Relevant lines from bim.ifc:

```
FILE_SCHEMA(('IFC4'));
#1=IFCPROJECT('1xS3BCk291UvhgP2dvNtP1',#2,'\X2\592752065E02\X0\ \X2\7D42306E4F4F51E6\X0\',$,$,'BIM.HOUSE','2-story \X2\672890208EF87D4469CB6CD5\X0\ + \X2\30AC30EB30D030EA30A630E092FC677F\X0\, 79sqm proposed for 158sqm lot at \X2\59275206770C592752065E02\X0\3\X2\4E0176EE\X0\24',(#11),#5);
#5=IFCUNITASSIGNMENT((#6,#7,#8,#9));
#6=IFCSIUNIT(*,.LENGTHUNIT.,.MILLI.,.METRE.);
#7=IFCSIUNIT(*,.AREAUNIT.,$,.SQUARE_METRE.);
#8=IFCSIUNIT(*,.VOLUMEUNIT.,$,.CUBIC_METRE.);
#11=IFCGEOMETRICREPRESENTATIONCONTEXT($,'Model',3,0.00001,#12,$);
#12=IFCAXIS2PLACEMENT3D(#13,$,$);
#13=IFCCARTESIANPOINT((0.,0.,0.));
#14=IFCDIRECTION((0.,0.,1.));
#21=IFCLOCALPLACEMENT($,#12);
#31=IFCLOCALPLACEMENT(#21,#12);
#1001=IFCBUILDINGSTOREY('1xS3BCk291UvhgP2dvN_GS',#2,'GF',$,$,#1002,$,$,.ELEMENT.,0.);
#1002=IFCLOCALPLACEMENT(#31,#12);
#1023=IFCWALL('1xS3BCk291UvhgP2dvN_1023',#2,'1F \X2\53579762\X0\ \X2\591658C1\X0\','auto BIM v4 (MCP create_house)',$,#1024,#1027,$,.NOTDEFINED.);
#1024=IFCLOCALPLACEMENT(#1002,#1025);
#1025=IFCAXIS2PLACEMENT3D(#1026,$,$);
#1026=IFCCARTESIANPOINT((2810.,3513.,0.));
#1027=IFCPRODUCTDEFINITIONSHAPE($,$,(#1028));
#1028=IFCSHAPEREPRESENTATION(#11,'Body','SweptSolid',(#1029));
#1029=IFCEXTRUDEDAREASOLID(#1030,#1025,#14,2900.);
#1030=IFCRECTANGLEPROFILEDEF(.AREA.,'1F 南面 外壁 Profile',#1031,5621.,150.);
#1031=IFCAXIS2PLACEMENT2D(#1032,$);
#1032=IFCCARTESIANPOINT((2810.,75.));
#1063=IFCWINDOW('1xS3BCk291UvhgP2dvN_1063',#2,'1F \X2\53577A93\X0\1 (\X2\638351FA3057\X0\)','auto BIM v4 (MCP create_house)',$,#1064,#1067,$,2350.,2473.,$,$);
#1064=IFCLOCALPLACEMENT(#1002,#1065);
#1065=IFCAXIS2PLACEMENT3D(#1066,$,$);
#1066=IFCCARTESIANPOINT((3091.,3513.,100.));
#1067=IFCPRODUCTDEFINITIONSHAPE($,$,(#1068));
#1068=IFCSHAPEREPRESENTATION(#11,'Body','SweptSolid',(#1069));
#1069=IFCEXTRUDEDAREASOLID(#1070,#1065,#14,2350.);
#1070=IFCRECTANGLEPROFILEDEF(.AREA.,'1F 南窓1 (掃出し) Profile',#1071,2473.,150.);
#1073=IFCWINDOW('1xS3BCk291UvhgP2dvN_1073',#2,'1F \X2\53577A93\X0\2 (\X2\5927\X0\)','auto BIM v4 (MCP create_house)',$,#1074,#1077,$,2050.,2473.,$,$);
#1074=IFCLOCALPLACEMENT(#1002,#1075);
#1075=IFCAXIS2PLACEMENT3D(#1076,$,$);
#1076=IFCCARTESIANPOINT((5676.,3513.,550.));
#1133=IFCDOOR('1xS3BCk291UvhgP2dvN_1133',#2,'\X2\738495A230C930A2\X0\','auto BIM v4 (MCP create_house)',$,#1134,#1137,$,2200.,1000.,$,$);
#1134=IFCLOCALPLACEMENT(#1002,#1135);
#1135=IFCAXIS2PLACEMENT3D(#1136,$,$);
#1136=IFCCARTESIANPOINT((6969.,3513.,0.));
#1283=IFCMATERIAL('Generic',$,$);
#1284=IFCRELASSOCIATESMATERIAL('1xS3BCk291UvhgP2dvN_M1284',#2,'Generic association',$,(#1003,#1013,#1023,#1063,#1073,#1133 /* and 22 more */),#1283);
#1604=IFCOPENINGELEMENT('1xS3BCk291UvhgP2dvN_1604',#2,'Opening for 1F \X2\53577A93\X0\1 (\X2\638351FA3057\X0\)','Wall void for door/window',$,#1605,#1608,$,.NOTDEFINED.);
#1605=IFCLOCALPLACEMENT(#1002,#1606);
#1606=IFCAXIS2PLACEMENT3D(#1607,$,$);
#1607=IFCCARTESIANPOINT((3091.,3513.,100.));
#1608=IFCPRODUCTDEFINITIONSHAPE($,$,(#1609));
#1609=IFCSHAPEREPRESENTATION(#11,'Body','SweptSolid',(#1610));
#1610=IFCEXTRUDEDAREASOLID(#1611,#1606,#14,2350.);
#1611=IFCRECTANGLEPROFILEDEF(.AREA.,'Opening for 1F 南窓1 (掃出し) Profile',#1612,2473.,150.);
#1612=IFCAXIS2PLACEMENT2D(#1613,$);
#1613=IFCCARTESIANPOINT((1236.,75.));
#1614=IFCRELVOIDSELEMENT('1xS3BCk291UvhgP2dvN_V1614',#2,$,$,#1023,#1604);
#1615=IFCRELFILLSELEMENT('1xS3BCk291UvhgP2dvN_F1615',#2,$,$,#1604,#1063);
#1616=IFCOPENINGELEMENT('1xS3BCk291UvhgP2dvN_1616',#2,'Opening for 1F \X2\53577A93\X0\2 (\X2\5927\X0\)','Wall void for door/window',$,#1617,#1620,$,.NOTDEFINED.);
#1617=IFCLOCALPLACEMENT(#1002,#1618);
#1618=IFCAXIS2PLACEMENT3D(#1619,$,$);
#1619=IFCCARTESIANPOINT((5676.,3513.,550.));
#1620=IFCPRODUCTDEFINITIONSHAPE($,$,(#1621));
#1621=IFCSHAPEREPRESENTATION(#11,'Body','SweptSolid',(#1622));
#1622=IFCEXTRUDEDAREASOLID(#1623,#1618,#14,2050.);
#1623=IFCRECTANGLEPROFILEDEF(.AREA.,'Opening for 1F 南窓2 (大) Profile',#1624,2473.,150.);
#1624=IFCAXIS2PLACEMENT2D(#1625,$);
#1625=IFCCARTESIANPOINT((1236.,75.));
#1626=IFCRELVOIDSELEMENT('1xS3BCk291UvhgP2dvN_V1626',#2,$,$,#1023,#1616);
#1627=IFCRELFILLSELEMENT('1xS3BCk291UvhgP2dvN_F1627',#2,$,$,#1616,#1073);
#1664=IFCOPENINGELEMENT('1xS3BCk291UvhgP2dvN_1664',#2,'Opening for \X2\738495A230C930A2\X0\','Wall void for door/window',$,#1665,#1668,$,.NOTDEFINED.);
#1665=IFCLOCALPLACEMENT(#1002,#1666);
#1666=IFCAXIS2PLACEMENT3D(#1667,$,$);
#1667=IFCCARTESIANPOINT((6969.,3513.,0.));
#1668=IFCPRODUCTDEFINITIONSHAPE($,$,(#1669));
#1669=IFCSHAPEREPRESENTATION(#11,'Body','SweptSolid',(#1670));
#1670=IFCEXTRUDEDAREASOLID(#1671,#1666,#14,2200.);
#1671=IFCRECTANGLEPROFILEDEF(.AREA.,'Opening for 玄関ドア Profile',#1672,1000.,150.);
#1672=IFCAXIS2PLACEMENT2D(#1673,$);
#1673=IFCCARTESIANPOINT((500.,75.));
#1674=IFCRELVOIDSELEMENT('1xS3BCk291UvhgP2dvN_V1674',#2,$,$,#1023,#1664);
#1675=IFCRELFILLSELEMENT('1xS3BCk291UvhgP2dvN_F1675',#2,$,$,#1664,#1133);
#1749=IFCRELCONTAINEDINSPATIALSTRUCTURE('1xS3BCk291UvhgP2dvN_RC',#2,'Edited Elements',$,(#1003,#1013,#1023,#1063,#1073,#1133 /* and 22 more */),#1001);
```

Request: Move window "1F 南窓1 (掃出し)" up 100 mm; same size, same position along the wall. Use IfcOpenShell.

```python
import numpy as np
import ifcopenshell
import ifcopenshell.api.geometry
import ifcopenshell.util.placement
import ifcopenshell.util.unit

model = ifcopenshell.open("bim.ifc")
unit_scale = ifcopenshell.util.unit.calculate_unit_scale(model)

window = model.by_id(1063)
opening = window.FillsVoids[0].RelatingOpeningElement
dz = 0.1 / unit_scale

shift = np.array([0.0, 0.0, dz])
# The window is not placed relative to its opening, so move both.
for product in (opening, window):
    matrix = ifcopenshell.util.placement.get_local_placement(product.ObjectPlacement)
    matrix[:3, 3] += shift
    ifcopenshell.api.geometry.edit_object_placement(model, product=product, matrix=matrix, is_si=False)

print(f"moved by {dz * unit_scale:+.3f} m")

model.write("bim_rev.ifc")
```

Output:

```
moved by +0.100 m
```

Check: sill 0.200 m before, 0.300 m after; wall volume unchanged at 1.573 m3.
